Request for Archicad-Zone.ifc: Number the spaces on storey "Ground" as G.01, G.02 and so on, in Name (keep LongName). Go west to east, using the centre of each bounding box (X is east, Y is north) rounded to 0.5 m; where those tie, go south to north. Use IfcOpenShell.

First a look at what the model holds.

```python
import ifcopenshell
import ifcopenshell.util.element
import ifcopenshell.util.placement

model = ifcopenshell.open("Archicad-Zone.ifc")
print(model.schema)
storey = next(s for s in model.by_type("IfcBuildingStorey") if s.Name == "Ground")
spaces = [e for e in ifcopenshell.util.element.get_decomposition(storey) if e.is_a("IfcSpace")]
for e in sorted(spaces, key=lambda e: e.id()):
    origin = ifcopenshell.util.placement.get_local_placement(e.ObjectPlacement)[:3, 3]
    print(e.id(), e.Name, e.LongName, origin.round(2) + 0.0, sep=" | ")
```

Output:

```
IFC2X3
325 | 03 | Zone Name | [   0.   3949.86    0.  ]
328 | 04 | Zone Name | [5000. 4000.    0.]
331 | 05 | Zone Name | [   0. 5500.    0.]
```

```python
import ifcopenshell
import ifcopenshell.geom
import ifcopenshell.util.element
import ifcopenshell.util.shape

model = ifcopenshell.open("Archicad-Zone.ifc")
settings = ifcopenshell.geom.settings()
settings.set("use-world-coords", True)


def centre(element):
    shape = ifcopenshell.geom.create_shape(settings, element)
    return ifcopenshell.util.shape.get_bbox_centroid(shape.geometry)


storey = next(s for s in model.by_type("IfcBuildingStorey") if s.Name == "Ground")
spaces = [e for e in ifcopenshell.util.element.get_decomposition(storey) if e.is_a("IfcSpace")]

# Insertion points can sit at a corner or the storey origin, so sort by the geometry (in metres).
centres = {e: centre(e) for e in spaces}
spaces.sort(key=lambda e: (round(centres[e][0] / 0.5), centres[e][1]))

for i, e in enumerate(spaces, start=1):
    number = f"G.{i:02d}"
    e.Name = number
    print(e.id(), number)

model.write("Archicad-Zone_updated.ifc")
```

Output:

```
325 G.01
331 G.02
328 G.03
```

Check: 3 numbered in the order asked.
